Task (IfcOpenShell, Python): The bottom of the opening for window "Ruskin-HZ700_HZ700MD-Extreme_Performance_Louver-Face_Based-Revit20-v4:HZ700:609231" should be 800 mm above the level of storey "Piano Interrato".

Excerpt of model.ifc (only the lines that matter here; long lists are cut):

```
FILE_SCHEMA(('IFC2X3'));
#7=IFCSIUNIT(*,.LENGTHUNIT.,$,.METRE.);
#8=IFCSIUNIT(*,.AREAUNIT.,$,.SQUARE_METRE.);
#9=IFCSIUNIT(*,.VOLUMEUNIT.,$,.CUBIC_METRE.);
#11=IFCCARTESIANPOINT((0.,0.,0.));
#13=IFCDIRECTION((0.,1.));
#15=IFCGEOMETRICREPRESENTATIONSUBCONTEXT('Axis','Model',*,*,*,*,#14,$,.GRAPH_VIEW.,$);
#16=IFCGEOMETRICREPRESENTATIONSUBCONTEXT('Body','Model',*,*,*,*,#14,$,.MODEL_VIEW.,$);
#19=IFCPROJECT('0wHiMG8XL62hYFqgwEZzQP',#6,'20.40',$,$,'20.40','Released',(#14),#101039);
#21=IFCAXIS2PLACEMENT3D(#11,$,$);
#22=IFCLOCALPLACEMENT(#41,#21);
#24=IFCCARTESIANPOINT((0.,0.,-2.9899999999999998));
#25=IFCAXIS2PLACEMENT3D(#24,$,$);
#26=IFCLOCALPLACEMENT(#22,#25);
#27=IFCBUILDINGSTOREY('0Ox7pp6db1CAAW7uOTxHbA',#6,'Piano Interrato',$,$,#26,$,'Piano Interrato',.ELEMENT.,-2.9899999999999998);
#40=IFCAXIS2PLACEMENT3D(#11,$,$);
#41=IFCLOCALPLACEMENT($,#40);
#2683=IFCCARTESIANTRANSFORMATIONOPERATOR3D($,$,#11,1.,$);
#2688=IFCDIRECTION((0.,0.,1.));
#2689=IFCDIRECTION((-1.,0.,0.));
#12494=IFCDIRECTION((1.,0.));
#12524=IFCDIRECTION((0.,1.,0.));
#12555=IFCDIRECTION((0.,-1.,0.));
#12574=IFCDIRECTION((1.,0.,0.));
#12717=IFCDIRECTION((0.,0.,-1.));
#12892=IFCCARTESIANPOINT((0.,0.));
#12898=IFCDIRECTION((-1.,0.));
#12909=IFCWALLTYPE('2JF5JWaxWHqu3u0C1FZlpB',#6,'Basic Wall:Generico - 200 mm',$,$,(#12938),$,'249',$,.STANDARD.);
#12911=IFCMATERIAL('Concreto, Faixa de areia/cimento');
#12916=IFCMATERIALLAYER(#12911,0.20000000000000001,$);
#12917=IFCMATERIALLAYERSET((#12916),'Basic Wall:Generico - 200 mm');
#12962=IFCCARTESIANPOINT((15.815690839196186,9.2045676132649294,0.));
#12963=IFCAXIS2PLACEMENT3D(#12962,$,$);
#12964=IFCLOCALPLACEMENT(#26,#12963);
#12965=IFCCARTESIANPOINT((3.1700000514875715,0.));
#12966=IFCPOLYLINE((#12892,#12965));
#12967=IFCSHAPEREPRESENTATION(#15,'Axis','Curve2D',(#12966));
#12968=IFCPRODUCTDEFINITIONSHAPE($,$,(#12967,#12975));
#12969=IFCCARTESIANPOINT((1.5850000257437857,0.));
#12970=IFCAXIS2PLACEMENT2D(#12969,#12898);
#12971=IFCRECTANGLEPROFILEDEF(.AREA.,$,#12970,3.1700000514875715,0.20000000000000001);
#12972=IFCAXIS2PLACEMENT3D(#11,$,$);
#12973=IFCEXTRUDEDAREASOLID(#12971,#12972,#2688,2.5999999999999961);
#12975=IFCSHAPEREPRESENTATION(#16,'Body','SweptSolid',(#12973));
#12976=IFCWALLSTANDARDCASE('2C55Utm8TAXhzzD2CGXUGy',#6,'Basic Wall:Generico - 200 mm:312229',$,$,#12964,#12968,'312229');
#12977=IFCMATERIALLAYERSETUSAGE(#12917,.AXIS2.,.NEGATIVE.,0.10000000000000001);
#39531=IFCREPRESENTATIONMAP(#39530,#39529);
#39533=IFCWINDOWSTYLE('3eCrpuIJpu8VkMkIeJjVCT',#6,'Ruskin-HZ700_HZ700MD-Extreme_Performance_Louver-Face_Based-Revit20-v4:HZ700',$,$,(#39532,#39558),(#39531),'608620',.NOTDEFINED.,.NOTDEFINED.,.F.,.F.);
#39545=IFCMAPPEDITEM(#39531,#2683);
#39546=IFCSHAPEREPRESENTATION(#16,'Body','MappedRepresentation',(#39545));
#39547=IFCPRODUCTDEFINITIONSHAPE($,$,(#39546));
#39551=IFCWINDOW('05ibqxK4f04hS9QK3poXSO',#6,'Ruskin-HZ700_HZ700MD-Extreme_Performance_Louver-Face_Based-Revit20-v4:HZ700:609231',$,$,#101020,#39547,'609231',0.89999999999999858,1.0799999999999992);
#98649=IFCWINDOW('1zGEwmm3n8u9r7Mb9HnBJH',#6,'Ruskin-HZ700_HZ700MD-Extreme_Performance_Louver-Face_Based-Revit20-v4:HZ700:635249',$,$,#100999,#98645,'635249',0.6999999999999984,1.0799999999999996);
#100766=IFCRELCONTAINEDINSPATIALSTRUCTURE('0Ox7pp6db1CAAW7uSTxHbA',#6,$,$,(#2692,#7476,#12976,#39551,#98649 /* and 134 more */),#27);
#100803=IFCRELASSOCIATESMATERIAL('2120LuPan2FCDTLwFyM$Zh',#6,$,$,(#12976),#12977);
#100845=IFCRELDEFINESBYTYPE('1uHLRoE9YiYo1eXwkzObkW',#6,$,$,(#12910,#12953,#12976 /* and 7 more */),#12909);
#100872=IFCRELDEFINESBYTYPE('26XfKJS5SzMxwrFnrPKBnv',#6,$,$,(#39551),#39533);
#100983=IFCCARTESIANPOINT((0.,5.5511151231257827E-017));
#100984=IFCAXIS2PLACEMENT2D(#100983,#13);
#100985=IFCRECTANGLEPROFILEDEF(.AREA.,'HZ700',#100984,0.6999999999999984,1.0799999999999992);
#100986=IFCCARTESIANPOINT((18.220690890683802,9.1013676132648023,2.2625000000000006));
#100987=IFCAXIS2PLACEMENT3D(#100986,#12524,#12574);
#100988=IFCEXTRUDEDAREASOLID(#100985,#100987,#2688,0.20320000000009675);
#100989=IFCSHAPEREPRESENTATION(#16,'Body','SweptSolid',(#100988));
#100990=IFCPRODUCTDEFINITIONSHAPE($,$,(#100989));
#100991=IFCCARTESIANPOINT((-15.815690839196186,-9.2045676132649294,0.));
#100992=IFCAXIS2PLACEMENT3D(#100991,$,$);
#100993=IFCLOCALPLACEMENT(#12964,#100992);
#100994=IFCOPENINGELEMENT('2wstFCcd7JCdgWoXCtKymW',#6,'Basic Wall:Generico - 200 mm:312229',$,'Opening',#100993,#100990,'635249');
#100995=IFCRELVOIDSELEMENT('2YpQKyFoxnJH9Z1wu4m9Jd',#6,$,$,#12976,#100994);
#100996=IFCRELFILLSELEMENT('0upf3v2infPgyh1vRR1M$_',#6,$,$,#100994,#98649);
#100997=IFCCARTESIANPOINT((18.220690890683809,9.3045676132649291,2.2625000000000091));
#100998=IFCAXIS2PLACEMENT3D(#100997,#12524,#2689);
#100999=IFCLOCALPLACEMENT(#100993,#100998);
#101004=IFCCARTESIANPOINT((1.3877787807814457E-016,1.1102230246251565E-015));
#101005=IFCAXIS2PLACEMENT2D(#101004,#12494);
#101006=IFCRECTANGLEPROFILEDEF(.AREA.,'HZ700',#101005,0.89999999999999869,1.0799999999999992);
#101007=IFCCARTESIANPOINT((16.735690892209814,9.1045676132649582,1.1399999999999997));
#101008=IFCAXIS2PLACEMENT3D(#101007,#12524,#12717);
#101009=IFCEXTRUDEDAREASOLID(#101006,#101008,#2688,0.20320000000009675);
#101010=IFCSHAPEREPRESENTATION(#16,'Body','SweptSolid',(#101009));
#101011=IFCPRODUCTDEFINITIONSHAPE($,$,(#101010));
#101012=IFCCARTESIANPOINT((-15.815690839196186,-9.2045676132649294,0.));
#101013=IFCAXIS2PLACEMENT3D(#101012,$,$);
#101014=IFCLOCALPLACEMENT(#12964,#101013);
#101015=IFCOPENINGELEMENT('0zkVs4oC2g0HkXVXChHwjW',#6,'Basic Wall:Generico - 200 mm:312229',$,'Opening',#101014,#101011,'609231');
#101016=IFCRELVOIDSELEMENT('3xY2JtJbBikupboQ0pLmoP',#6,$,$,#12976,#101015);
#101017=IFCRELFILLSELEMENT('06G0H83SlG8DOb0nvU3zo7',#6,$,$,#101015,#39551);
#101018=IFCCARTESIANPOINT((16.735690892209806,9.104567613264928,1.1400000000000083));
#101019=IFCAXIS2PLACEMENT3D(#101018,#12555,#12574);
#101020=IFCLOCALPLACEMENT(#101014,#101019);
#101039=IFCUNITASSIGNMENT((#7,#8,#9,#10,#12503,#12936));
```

```python
import numpy as np
import ifcopenshell
import ifcopenshell.api.geometry
import ifcopenshell.geom
import ifcopenshell.util.element
import ifcopenshell.util.placement
import ifcopenshell.util.shape
import ifcopenshell.util.unit

model = ifcopenshell.open("model.ifc")
unit_scale = ifcopenshell.util.unit.calculate_unit_scale(model)

window = model.by_guid("05ibqxK4f04hS9QK3poXSO")
opening = window.FillsVoids[0].RelatingOpeningElement
storey = ifcopenshell.util.element.get_container(window, ifc_class="IfcBuildingStorey")
level = ifcopenshell.util.placement.get_local_placement(storey.ObjectPlacement)[2, 3]

# The opening's origin need not be at the sill, so measure its lowest point.
shape = ifcopenshell.geom.create_shape(ifcopenshell.geom.settings(), opening)
bottom = ifcopenshell.util.shape.get_shape_bottom_elevation(shape, shape.geometry) / unit_scale
dz = level + 0.8 / unit_scale - bottom

shift = np.array([0.0, 0.0, dz])
# The window is placed relative to its opening, so it follows when the opening moves.
matrix = ifcopenshell.util.placement.get_local_placement(opening.ObjectPlacement)
matrix[:3, 3] += shift
ifcopenshell.api.geometry.edit_object_placement(
    model, product=opening, matrix=matrix, is_si=False, should_transform_children=True
)

print(f"moved by {dz * unit_scale:+.3f} m")

model.write("model-out.ifc")
```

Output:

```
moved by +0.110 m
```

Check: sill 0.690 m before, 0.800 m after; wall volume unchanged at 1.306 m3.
